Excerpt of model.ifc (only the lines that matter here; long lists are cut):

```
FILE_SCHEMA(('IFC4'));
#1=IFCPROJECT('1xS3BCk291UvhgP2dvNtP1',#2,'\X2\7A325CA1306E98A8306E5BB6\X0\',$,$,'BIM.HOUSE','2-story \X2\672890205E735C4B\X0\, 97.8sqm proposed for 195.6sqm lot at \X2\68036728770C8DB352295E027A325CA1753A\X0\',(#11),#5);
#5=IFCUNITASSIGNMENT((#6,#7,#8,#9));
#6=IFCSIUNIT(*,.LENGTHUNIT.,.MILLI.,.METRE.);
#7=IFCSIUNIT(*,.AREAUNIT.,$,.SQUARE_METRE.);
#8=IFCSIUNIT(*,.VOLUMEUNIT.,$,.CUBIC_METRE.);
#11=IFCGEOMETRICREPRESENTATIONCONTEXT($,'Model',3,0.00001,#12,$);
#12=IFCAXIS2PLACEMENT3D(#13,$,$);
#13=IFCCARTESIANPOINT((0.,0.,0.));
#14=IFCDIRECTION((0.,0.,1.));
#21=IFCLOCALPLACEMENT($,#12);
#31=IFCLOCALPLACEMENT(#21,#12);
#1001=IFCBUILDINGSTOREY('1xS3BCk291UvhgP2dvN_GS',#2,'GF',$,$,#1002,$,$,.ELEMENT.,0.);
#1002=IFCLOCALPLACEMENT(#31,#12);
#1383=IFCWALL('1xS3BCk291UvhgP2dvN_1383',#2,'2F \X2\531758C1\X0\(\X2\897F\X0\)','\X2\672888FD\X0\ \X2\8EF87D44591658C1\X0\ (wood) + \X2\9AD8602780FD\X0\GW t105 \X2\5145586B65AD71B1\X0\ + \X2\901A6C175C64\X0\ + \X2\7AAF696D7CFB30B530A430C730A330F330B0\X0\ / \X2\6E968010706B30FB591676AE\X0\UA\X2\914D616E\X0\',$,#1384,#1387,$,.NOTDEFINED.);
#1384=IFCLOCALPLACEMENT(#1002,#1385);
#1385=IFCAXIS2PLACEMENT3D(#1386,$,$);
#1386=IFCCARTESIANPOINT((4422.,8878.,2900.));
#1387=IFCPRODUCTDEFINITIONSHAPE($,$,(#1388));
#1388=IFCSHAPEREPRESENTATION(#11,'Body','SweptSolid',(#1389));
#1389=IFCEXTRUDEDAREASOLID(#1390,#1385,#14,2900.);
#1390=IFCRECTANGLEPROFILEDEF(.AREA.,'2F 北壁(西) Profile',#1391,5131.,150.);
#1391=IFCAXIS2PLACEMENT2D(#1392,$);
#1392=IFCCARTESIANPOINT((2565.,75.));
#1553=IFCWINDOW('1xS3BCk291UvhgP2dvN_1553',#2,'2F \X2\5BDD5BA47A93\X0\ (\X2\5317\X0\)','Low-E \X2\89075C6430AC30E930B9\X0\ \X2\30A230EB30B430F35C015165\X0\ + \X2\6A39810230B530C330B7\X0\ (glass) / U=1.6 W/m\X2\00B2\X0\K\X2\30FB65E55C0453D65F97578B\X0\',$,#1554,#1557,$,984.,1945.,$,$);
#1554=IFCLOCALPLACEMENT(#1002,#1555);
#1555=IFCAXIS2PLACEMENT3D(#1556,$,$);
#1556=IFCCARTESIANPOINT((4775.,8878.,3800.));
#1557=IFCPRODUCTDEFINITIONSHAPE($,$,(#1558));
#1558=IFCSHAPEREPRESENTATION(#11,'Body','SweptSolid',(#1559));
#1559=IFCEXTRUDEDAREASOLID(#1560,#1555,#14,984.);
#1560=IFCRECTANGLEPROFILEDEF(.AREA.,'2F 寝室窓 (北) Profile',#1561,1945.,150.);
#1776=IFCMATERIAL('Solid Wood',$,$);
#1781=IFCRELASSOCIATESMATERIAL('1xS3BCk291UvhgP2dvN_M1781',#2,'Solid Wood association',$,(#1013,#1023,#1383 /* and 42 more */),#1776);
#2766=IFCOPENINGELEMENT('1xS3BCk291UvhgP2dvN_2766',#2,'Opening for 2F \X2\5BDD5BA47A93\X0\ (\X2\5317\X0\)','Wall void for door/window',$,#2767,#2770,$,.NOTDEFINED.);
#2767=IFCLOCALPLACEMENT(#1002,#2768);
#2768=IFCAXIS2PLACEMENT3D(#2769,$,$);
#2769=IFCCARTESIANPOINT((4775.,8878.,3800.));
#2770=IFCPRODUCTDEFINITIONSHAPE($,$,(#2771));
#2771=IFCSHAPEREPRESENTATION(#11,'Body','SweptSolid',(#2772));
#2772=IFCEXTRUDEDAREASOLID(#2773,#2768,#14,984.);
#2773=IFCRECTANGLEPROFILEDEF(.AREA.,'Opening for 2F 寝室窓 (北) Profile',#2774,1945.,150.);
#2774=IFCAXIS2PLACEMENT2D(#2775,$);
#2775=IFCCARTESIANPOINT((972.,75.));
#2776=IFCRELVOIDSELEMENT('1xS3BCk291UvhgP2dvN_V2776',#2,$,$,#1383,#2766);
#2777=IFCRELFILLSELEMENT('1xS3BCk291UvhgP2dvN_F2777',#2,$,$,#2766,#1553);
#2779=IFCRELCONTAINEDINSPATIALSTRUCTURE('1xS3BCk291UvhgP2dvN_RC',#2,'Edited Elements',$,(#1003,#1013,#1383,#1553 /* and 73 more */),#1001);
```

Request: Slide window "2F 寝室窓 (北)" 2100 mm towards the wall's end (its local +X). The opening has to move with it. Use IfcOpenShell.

```python
import ifcopenshell
import ifcopenshell.api.geometry
import ifcopenshell.util.placement
import ifcopenshell.util.unit

model = ifcopenshell.open("model.ifc")
unit_scale = ifcopenshell.util.unit.calculate_unit_scale(model)

window = model.by_guid("1xS3BCk291UvhgP2dvN_1553")
opening = window.FillsVoids[0].RelatingOpeningElement
wall = opening.VoidsElements[0].RelatingBuildingElement

wall_matrix = ifcopenshell.util.placement.get_local_placement(wall.ObjectPlacement)
shift = wall_matrix[:3, 0] * 2.1 / unit_scale
before = ifcopenshell.util.placement.get_local_placement(window.ObjectPlacement)[:3, 3].copy()

# The window is not placed relative to its opening, so move both.
for product in (opening, window):
    matrix = ifcopenshell.util.placement.get_local_placement(product.ObjectPlacement)
    matrix[:3, 3] += shift
    ifcopenshell.api.geometry.edit_object_placement(model, product=product, matrix=matrix, is_si=False)

after = ifcopenshell.util.placement.get_local_placement(window.ObjectPlacement)[:3, 3]
print("window moved by", (after - before).round(3) + 0.0)

model.write("model_rev.ifc")
```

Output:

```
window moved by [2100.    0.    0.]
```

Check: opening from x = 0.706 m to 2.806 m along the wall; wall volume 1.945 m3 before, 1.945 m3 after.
